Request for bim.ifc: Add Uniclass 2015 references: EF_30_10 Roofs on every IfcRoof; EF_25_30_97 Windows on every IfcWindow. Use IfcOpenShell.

First a look at what the model holds.

```python
import ifcopenshell

model = ifcopenshell.open("bim.ifc")
print(model.schema)
print("classifications:", [c.Name for c in model.by_type("IfcClassification")])
for ifc_class in ("IfcDoor", "IfcRoof", "IfcStair", "IfcWall", "IfcWindow"):
    print(ifc_class, len(model.by_type(ifc_class)))
```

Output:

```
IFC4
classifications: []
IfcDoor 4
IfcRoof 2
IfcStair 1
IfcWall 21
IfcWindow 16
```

```python
import ifcopenshell
import ifcopenshell.api.classification

model = ifcopenshell.open("bim.ifc")

system = ifcopenshell.api.classification.add_classification(model, classification="Uniclass 2015")

codes = {
    "IfcRoof": ("EF_30_10", "Roofs"),
    "IfcWindow": ("EF_25_30_97", "Windows"),
}
for ifc_class, (code, name) in codes.items():
    products = model.by_type(ifc_class)
    ifcopenshell.api.classification.add_reference(
        model, products=products, classification=system, identification=code, name=name
    )
    print(code, len(products))

model.write("bim_v2.ifc")
```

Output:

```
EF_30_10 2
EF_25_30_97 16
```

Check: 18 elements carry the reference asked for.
